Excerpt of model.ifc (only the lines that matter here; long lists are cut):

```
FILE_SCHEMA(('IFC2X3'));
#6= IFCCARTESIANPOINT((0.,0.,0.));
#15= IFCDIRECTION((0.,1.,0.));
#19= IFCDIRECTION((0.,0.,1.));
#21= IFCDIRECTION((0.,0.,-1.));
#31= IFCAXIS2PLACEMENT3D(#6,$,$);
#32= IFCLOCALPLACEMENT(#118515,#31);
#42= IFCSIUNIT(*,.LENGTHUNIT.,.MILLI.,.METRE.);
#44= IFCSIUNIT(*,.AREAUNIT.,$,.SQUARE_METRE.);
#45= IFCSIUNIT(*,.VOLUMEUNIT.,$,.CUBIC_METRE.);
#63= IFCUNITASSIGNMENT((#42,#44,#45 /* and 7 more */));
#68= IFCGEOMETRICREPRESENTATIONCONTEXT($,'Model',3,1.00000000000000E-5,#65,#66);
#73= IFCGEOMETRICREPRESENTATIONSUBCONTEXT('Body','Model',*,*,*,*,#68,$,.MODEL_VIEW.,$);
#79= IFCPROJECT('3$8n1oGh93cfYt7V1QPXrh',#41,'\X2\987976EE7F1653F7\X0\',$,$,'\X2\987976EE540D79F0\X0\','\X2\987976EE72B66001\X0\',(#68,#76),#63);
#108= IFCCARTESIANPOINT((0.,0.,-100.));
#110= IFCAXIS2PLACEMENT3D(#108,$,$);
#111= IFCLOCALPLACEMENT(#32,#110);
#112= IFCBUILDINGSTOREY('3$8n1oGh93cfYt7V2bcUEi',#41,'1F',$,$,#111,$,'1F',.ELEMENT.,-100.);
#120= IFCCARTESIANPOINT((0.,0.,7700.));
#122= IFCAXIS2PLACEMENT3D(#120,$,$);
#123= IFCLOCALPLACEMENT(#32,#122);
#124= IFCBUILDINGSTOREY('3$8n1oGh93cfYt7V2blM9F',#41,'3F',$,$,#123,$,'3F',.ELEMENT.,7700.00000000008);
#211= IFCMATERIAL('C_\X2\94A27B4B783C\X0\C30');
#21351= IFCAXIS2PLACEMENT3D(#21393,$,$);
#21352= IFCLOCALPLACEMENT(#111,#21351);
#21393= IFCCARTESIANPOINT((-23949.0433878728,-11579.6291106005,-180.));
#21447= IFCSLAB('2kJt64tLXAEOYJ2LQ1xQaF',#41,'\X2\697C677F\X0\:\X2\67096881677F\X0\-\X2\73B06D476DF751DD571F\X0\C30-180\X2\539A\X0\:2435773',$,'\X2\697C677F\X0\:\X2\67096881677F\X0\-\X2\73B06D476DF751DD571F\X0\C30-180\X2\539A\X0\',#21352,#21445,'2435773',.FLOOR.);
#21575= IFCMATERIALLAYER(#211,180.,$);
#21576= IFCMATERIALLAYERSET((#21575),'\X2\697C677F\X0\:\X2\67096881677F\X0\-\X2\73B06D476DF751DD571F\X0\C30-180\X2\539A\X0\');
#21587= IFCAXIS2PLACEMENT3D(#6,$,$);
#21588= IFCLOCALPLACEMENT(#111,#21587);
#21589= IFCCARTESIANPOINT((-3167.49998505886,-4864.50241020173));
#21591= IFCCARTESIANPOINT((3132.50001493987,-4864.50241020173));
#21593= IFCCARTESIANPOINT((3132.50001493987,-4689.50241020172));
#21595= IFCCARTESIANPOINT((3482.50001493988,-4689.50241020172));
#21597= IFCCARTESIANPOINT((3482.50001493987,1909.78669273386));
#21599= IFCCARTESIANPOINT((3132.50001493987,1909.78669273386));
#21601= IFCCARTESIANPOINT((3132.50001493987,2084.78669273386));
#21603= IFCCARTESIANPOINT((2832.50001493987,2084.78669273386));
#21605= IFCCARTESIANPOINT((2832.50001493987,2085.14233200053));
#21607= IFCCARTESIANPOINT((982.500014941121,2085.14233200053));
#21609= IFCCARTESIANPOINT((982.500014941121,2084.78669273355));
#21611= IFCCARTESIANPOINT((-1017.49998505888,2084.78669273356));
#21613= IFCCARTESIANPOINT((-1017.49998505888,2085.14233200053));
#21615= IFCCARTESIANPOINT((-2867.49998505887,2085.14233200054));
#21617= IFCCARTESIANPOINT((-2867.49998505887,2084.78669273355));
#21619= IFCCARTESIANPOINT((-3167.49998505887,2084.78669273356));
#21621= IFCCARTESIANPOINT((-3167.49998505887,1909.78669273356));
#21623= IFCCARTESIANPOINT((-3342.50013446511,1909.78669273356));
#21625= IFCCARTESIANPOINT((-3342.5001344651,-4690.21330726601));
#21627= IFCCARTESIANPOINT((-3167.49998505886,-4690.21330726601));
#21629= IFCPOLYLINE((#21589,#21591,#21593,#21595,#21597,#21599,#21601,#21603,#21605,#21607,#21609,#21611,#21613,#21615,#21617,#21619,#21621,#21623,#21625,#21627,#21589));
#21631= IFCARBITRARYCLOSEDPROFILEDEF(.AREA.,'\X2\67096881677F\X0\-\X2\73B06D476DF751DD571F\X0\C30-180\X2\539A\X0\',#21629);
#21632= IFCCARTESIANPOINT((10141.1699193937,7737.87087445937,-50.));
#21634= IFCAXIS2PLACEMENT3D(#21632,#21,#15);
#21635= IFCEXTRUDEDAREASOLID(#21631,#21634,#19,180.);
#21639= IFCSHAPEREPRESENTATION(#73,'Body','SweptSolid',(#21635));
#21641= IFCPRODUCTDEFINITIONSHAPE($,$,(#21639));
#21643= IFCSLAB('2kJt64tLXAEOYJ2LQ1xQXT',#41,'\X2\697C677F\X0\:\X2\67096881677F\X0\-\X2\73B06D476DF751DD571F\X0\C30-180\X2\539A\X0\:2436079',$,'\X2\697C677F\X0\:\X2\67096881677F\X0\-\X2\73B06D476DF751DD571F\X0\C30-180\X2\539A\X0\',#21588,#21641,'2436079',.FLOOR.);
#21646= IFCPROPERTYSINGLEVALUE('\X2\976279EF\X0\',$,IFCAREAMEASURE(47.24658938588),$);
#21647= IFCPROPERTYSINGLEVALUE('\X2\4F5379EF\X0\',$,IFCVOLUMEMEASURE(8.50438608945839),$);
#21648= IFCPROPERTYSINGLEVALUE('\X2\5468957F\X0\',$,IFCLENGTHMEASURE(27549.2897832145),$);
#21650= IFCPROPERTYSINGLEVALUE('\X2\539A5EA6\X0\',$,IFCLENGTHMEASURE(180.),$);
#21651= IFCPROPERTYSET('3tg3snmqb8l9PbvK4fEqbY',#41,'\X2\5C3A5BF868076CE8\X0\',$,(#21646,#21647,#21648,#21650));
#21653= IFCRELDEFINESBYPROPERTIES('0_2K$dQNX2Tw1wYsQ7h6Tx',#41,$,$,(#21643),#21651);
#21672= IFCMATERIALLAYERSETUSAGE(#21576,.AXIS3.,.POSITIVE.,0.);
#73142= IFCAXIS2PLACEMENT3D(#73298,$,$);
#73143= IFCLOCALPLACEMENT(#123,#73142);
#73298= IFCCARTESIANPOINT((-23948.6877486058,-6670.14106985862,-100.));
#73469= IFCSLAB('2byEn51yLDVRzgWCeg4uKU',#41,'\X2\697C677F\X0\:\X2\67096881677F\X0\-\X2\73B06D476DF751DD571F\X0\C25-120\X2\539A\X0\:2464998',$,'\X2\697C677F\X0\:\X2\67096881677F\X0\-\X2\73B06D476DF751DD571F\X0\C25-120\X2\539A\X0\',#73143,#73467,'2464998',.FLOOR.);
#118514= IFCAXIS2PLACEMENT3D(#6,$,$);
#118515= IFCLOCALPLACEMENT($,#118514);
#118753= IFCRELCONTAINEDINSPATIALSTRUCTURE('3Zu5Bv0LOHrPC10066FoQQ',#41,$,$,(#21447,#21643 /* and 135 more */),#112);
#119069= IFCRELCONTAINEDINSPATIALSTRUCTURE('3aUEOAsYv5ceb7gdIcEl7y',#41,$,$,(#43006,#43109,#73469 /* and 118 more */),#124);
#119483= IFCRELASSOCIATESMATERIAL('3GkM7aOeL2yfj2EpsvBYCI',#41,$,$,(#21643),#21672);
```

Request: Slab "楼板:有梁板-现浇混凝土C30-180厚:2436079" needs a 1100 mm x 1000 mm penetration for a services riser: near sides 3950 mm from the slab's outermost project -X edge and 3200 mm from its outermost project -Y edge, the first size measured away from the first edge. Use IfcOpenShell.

```python
import numpy as np
import ifcopenshell
import ifcopenshell.api.feature
import ifcopenshell.api.geometry
import ifcopenshell.api.pset
import ifcopenshell.api.root
import ifcopenshell.geom
import ifcopenshell.util.element
import ifcopenshell.util.placement
import ifcopenshell.util.representation
import ifcopenshell.util.shape
import ifcopenshell.util.unit

model = ifcopenshell.open("model.ifc")
unit_scale = ifcopenshell.util.unit.calculate_unit_scale(model)
area_scale = ifcopenshell.util.unit.calculate_unit_scale(model, "AREAUNIT")
volume_scale = ifcopenshell.util.unit.calculate_unit_scale(model, "VOLUMEUNIT")
settings = ifcopenshell.geom.settings()


def volume(element):
    """Net volume in cubic metres, openings subtracted."""
    shape = ifcopenshell.geom.create_shape(settings, element)
    return ifcopenshell.util.shape.get_volume(shape.geometry)


slab = model.by_guid("2kJt64tLXAEOYJ2LQ1xQXT")
before = volume(slab)

# Extent in the slab's own axes, in metres. The edges named are its -X and -Y sides.
slab_shape = ifcopenshell.geom.create_shape(settings, slab)
vertices = ifcopenshell.util.shape.get_vertices(slab_shape.geometry)
x_min, y_min, bottom = vertices.min(axis=0)
top = vertices[:, 2].max()

opening = ifcopenshell.api.root.create_entity(model, ifc_class="IfcOpeningElement", name="Services riser opening")
context = ifcopenshell.util.representation.get_context(model, "Model", "Body", "MODEL_VIEW")
width, depth = 1.1, 1
outline = [(0.0, 0.0), (width, 0.0), (width, depth), (0.0, depth), (0.0, 0.0)]
# Overshoot both faces by 50 mm so the cut is clean.
shape = ifcopenshell.api.geometry.add_slab_representation(
    model, context=context, depth=top - bottom + 0.1, polyline=outline
)
ifcopenshell.api.geometry.assign_representation(model, product=opening, representation=shape)

matrix = ifcopenshell.util.placement.get_local_placement(slab.ObjectPlacement)
matrix[:, 3] = matrix @ np.append(np.array([x_min + 3.95, y_min + 3.2, bottom - 0.05]) / unit_scale, 1.0)
ifcopenshell.api.geometry.edit_object_placement(model, product=opening, matrix=matrix, is_si=False)
ifcopenshell.api.feature.add_feature(model, feature=opening, element=slab)

after = volume(slab)

# Update the slab's stored quantities.
pset = model.by_id(ifcopenshell.util.element.get_pset(slab, "尺寸标注", should_inherit=False)["id"])
ifcopenshell.api.pset.edit_pset(model, pset=pset, properties={
    "面积": model.create_entity("IfcAreaMeasure", after / (top - bottom) / area_scale),
    "体积": model.create_entity("IfcVolumeMeasure", after / volume_scale),
})

print(f"slab volume {before:.3f} -> {after:.3f} m3")

model.write("model_rev.ifc")
```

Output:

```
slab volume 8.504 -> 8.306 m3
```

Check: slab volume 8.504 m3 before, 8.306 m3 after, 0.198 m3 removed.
